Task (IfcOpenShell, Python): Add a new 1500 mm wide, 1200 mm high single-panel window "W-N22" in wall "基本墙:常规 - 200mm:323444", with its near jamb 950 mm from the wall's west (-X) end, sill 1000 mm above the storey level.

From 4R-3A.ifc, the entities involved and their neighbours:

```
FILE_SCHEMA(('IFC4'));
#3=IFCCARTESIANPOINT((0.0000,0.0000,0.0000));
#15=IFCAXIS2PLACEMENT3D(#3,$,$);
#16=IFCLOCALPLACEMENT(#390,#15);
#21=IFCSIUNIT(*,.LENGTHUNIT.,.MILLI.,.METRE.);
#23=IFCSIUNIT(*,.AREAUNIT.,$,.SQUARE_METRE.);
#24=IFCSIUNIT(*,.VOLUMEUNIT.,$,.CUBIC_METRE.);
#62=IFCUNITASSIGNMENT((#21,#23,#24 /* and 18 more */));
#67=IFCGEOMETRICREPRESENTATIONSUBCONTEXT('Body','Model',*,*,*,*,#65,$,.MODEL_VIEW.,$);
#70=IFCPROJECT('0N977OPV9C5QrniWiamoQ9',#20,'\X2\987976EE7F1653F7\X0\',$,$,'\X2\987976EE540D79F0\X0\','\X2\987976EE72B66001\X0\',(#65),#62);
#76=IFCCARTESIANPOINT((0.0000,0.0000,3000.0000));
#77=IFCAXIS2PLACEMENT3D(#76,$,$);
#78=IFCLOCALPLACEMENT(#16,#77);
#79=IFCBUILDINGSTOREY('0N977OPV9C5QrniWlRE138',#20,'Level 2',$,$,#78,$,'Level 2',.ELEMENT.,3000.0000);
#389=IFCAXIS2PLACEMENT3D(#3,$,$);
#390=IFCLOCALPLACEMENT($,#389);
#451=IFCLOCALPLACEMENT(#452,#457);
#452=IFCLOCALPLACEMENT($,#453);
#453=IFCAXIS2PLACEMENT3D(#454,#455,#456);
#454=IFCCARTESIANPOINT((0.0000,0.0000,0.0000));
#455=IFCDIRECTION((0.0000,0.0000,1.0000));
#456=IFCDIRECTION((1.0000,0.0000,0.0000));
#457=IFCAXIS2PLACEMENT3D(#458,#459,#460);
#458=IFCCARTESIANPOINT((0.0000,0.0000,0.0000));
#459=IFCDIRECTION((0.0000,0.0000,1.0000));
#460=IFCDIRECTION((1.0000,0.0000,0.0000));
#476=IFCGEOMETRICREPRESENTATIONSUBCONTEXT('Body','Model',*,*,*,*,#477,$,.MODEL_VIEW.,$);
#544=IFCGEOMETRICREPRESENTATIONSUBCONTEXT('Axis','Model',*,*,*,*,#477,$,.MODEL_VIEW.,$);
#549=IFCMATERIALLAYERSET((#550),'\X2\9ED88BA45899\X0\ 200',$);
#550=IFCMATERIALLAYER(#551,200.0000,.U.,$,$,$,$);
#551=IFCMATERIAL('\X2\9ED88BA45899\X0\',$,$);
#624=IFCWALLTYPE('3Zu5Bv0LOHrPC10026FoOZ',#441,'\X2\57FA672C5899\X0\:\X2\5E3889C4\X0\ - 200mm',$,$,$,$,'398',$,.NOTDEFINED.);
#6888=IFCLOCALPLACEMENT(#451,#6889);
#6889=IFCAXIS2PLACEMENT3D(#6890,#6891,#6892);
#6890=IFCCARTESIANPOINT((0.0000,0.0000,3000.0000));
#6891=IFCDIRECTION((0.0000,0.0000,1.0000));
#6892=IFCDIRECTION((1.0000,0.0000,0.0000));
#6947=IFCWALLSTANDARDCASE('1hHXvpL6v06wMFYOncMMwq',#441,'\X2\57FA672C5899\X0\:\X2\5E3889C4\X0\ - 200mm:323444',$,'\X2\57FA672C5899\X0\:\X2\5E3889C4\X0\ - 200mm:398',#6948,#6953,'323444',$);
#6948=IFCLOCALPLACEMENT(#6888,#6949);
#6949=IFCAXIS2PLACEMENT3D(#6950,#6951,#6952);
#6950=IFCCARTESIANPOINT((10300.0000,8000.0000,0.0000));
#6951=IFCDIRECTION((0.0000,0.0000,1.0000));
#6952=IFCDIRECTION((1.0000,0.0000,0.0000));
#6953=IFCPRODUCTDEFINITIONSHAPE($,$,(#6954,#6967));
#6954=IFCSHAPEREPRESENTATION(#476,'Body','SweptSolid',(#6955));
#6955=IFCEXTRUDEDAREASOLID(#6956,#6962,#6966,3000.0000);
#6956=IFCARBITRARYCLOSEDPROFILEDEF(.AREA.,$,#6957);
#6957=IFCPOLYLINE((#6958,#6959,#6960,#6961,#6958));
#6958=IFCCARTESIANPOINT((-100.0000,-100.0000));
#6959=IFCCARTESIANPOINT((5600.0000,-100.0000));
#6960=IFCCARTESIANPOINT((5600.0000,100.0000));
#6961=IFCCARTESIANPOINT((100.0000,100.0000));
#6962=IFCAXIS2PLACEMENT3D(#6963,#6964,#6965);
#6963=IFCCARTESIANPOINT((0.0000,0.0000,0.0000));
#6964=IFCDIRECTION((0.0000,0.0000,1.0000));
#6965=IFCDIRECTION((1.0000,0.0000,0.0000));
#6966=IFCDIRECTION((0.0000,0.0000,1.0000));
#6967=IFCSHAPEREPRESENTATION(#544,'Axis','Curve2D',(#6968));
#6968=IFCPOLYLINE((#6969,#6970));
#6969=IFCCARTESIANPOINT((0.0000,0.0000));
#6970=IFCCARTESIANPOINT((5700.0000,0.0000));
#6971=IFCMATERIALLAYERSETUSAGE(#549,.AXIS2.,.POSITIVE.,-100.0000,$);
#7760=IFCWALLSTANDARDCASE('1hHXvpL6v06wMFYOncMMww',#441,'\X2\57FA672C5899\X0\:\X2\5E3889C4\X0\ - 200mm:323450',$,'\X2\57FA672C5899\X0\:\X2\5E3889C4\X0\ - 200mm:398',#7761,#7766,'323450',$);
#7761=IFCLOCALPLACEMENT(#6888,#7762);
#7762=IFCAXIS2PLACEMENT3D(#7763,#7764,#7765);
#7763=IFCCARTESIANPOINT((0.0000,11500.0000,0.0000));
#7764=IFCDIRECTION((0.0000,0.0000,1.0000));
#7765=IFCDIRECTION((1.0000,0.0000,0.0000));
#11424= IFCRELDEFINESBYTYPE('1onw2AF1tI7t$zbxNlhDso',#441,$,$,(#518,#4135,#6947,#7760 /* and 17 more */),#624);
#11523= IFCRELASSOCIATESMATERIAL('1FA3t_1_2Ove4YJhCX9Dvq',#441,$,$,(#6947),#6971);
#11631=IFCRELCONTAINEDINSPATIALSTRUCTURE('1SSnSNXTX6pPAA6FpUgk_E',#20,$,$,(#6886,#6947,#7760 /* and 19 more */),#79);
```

```python
import numpy as np
import ifcopenshell
import ifcopenshell.api.feature
import ifcopenshell.api.geometry
import ifcopenshell.api.root
import ifcopenshell.api.spatial
import ifcopenshell.geom
import ifcopenshell.util.element
import ifcopenshell.util.placement
import ifcopenshell.util.representation
import ifcopenshell.util.shape
import ifcopenshell.util.unit

model = ifcopenshell.open("4R-3A.ifc")
unit_scale = ifcopenshell.util.unit.calculate_unit_scale(model)
settings = ifcopenshell.geom.settings()


def volume(element):
    """Net volume in cubic metres, openings subtracted."""
    shape = ifcopenshell.geom.create_shape(settings, element)
    return ifcopenshell.util.shape.get_volume(shape.geometry)


wall = model.by_guid("1hHXvpL6v06wMFYOncMMwq")
storey = ifcopenshell.util.element.get_container(wall, ifc_class="IfcBuildingStorey")
context = ifcopenshell.util.representation.get_context(model, "Model", "Body", "MODEL_VIEW")
before = volume(wall)

width, height, from_end, sill = 1.5, 1.2, 0.95, 1  # metres

# The wall runs along its own X axis, and the end named is its -X end.
wall_shape = ifcopenshell.geom.create_shape(settings, wall)
x, y, z = ifcopenshell.util.shape.get_vertices(wall_shape.geometry).T
start = x.min() + from_end
face, thickness = float(y.min()), float(y.max() - y.min())
wall_matrix = ifcopenshell.util.placement.get_local_placement(wall.ObjectPlacement)
level = ifcopenshell.util.placement.get_local_placement(storey.ObjectPlacement)[2, 3]


def in_wall(x, y):
    """Placement at x, y metres in the wall's axes, at sill height."""
    matrix = wall_matrix.copy()
    matrix[:, 3] = wall_matrix @ np.array([x / unit_scale, y / unit_scale, 0.0, 1.0])
    matrix[2, 3] = level + sill / unit_scale
    return matrix


# Opening: a box that overshoots both wall faces by 50 mm.
opening = ifcopenshell.api.root.create_entity(model, ifc_class="IfcOpeningElement", predefined_type="OPENING")
box = ifcopenshell.api.geometry.add_wall_representation(
    model, context=context, length=width, height=height, thickness=thickness + 0.1
)
ifcopenshell.api.geometry.assign_representation(model, product=opening, representation=box)
ifcopenshell.api.geometry.edit_object_placement(model, product=opening, matrix=in_wall(start, face - 0.05), is_si=False)
ifcopenshell.api.feature.add_feature(model, feature=opening, element=wall)

window = ifcopenshell.api.root.create_entity(model, ifc_class="IfcWindow", name="W-N22", predefined_type="WINDOW")
window.OverallWidth, window.OverallHeight = width / unit_scale, height / unit_scale
window.PartitioningType = "SINGLE_PANEL"
body = ifcopenshell.api.geometry.add_window_representation(
    model,
    context=context,
    overall_width=window.OverallWidth,
    overall_height=window.OverallHeight,
    partition_type="SINGLE_PANEL",
)
ifcopenshell.api.geometry.assign_representation(model, product=window, representation=body)
ifcopenshell.api.spatial.assign_container(model, products=[window], relating_structure=storey)
ifcopenshell.api.feature.add_filling(model, opening=opening, element=window)

# Centre the window in the wall's thickness.
ifcopenshell.api.geometry.edit_object_placement(model, product=window, matrix=in_wall(start, face), is_si=False)
window_shape = ifcopenshell.geom.create_shape(settings, window)
depth = ifcopenshell.util.shape.get_vertices(window_shape.geometry)[:, 1]
offset = face + thickness / 2 - (depth.min() + depth.max()) / 2
ifcopenshell.api.geometry.edit_object_placement(model, product=window, matrix=in_wall(start, offset), is_si=False)

after = volume(wall)

print(f"wall volume {before:.3f} -> {after:.3f} m3")

model.write("4R-3A_v2.ifc")
```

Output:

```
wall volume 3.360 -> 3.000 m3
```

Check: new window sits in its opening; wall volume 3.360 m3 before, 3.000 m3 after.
